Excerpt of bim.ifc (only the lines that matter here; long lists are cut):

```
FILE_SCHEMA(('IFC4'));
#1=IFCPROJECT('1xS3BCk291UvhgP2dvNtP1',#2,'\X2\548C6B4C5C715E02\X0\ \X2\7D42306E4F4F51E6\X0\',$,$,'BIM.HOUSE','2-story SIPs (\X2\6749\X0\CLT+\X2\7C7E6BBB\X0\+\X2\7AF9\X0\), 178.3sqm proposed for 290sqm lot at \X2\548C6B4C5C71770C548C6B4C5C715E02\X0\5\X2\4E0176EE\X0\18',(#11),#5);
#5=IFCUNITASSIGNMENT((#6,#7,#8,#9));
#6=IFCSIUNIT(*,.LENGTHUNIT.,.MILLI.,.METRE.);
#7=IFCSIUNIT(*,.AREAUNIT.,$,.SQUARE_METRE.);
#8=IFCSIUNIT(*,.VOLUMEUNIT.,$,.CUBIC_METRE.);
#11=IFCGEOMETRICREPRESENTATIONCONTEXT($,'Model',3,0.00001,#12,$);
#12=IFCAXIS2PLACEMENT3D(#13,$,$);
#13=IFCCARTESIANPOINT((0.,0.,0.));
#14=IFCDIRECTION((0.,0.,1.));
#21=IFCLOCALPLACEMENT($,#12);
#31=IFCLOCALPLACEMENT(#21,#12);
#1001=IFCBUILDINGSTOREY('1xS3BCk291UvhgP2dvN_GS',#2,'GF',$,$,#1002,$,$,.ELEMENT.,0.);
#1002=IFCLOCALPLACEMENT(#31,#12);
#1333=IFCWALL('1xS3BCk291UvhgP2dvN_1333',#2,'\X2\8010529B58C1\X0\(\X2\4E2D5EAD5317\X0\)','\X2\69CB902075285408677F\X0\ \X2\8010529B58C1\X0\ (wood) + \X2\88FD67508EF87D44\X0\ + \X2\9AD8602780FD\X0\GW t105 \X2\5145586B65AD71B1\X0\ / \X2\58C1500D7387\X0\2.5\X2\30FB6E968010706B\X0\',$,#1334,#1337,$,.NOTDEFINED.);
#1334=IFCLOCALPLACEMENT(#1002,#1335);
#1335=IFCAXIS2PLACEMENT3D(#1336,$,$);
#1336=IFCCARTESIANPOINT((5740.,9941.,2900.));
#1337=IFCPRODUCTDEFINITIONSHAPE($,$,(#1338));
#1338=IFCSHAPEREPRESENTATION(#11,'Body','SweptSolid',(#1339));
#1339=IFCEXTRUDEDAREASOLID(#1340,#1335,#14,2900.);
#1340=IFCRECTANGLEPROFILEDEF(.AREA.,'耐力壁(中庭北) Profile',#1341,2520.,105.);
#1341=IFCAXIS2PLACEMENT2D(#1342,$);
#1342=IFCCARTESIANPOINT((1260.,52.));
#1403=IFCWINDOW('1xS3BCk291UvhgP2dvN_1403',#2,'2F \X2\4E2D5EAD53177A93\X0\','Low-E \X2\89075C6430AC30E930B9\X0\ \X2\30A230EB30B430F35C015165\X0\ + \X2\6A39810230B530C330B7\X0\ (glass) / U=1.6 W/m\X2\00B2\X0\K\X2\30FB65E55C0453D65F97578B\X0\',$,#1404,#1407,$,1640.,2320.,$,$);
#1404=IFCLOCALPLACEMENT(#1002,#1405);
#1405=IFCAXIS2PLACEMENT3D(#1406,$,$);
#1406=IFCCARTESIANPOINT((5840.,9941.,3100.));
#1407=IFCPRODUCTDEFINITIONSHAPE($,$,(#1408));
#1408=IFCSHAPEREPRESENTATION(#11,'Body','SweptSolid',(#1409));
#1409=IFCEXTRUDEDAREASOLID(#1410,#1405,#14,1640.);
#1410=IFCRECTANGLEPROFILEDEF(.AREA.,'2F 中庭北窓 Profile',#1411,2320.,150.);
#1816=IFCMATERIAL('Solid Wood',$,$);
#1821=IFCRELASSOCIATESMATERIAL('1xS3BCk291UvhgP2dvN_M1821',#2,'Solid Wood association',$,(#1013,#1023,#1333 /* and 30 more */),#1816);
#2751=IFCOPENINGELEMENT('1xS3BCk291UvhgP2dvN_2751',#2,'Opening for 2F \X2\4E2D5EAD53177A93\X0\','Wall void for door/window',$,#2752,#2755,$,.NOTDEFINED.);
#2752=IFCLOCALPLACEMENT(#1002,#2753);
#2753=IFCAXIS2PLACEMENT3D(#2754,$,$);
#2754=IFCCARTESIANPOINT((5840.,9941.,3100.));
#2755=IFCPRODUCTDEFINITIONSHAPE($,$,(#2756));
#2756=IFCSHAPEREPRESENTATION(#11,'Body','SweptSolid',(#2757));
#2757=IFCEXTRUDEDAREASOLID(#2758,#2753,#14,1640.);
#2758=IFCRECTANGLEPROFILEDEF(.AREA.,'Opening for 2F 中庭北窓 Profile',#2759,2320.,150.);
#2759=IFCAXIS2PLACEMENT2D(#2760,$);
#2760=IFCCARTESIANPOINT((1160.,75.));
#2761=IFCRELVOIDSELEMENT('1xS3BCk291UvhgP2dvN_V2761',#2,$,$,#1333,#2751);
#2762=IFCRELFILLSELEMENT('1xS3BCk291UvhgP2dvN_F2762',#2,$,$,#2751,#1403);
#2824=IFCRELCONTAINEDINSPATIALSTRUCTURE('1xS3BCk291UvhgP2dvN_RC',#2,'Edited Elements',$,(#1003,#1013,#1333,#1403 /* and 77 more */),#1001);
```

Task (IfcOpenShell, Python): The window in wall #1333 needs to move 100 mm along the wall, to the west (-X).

```python
import ifcopenshell
import ifcopenshell.api.geometry
import ifcopenshell.util.placement

model = ifcopenshell.open("bim.ifc")

window = model.by_guid("1xS3BCk291UvhgP2dvN_1403")
opening = window.FillsVoids[0].RelatingOpeningElement
wall = opening.VoidsElements[0].RelatingBuildingElement

wall_matrix = ifcopenshell.util.placement.get_local_placement(wall.ObjectPlacement)
shift = wall_matrix[:3, 0] * -100.0
before = ifcopenshell.util.placement.get_local_placement(window.ObjectPlacement)[:3, 3].copy()

# The window is not placed relative to its opening, so move both.
for product in (opening, window):
    matrix = ifcopenshell.util.placement.get_local_placement(product.ObjectPlacement)
    matrix[:3, 3] += shift
    ifcopenshell.api.geometry.edit_object_placement(model, product=product, matrix=matrix, is_si=False)

after = ifcopenshell.util.placement.get_local_placement(window.ObjectPlacement)[:3, 3]
print("window moved by", (after - before).round(3) + 0.0)

model.write("bim_v2.ifc")
```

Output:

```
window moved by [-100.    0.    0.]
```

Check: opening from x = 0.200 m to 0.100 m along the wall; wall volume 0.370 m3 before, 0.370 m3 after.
